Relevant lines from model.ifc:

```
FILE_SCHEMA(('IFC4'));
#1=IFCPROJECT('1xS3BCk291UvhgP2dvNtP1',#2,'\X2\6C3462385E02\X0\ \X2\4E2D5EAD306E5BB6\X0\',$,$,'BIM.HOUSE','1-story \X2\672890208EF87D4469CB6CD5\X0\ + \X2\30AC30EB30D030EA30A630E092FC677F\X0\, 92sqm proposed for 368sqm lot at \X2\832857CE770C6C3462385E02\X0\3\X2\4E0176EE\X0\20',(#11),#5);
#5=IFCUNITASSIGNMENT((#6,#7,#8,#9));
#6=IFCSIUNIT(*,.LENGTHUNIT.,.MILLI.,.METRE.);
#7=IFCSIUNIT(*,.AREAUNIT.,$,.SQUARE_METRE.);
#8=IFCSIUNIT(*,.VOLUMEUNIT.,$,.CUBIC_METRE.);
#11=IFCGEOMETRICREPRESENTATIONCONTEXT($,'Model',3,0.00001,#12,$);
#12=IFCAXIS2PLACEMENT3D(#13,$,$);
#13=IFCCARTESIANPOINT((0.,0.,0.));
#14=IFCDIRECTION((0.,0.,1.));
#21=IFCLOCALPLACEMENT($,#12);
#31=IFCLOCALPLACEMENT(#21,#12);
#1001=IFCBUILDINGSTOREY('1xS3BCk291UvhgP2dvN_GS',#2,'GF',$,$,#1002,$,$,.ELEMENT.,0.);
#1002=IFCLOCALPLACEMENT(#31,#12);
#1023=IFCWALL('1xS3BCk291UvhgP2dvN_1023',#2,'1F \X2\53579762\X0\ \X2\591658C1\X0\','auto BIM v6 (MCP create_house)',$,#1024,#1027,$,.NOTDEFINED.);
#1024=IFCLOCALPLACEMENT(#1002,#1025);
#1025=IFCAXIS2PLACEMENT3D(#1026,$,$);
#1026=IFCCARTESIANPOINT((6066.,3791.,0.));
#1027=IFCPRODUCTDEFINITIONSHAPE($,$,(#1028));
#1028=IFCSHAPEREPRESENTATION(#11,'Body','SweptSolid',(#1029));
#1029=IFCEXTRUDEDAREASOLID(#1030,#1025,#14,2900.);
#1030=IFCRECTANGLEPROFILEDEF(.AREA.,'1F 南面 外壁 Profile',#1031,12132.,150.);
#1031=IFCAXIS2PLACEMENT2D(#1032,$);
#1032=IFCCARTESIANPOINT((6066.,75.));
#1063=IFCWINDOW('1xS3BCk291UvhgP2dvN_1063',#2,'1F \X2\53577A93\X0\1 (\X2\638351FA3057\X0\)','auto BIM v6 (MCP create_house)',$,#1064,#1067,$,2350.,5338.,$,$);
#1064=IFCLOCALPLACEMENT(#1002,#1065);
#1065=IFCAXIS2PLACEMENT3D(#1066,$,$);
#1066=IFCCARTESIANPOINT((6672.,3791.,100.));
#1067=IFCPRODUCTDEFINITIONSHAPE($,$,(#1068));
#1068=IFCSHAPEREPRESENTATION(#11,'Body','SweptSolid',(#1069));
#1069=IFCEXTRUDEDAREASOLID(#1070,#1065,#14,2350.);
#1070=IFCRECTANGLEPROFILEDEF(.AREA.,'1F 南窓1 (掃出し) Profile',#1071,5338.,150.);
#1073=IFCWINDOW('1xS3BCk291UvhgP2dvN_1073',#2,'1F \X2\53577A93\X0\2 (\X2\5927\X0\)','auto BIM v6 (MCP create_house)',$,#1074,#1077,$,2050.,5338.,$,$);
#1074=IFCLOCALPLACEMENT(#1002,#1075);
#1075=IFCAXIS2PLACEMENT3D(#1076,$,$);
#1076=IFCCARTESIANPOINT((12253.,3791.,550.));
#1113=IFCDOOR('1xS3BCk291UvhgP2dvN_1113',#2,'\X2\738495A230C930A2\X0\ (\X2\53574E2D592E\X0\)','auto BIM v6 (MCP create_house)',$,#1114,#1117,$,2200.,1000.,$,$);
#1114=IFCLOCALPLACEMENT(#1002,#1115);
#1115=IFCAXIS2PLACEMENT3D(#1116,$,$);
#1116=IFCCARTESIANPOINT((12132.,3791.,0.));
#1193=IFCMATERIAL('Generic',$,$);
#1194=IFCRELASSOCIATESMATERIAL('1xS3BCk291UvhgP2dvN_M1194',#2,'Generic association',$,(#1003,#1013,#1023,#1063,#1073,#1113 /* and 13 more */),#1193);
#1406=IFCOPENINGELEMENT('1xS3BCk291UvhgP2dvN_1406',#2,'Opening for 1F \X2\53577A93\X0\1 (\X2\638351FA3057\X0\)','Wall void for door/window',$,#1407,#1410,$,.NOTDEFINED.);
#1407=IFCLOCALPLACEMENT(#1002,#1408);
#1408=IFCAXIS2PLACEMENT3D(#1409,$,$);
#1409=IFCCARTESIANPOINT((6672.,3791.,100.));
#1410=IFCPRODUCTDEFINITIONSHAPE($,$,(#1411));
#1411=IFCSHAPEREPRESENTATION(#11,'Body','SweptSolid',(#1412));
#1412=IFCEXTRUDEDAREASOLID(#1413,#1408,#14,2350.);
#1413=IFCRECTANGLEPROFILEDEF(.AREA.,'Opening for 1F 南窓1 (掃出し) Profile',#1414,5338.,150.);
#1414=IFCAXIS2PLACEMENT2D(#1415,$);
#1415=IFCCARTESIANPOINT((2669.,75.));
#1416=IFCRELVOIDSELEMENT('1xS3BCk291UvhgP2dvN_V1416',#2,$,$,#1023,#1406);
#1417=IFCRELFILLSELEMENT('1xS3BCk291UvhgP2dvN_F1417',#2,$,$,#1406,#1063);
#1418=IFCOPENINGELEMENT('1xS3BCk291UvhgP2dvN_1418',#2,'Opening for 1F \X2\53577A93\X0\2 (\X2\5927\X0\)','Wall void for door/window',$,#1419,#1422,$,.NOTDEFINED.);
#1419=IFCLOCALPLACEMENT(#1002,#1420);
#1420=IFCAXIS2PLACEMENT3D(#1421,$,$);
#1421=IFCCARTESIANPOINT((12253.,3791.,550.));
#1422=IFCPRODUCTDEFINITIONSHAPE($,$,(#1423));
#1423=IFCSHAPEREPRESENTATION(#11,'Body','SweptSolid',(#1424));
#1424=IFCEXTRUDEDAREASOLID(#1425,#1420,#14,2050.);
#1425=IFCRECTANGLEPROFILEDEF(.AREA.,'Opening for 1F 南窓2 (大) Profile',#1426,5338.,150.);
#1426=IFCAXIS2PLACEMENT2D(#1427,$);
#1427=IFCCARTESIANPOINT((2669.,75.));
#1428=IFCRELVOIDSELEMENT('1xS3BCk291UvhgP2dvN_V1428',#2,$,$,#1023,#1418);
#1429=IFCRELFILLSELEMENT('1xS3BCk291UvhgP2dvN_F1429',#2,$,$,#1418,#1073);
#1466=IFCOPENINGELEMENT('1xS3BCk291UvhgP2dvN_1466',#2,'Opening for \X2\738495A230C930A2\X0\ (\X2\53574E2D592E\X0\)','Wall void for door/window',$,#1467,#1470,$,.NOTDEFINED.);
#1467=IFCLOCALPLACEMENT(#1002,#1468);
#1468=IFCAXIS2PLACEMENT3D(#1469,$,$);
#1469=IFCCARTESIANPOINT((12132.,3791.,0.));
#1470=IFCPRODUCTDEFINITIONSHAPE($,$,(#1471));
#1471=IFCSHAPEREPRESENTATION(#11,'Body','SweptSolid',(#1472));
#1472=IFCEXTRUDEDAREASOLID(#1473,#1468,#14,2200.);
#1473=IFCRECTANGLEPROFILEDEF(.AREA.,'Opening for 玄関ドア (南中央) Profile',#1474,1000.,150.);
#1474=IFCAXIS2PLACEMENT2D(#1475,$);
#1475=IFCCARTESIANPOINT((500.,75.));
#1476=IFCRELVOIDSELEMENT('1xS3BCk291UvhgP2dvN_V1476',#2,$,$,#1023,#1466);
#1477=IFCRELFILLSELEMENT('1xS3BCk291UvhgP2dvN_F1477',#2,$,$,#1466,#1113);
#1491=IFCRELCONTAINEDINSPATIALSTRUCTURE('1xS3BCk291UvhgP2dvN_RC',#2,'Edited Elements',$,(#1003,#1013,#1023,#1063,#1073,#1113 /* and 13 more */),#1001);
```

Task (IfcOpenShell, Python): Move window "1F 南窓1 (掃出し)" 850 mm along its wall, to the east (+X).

```python
import ifcopenshell
import ifcopenshell.api.geometry
import ifcopenshell.util.placement
import ifcopenshell.util.unit

model = ifcopenshell.open("model.ifc")
unit_scale = ifcopenshell.util.unit.calculate_unit_scale(model)

window = model.by_id(1063)
opening = window.FillsVoids[0].RelatingOpeningElement
wall = opening.VoidsElements[0].RelatingBuildingElement

wall_matrix = ifcopenshell.util.placement.get_local_placement(wall.ObjectPlacement)
shift = wall_matrix[:3, 0] * 0.85 / unit_scale
before = ifcopenshell.util.placement.get_local_placement(window.ObjectPlacement)[:3, 3].copy()

# The window is not placed relative to its opening, so move both.
for product in (opening, window):
    matrix = ifcopenshell.util.placement.get_local_placement(product.ObjectPlacement)
    matrix[:3, 3] += shift
    ifcopenshell.api.geometry.edit_object_placement(model, product=product, matrix=matrix, is_si=False)

after = ifcopenshell.util.placement.get_local_placement(window.ObjectPlacement)[:3, 3]
print("window moved by", (after - before).round(3) + 0.0)

model.write("model_updated.ifc")
```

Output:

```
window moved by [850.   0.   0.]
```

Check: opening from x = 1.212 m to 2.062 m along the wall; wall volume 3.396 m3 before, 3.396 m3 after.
